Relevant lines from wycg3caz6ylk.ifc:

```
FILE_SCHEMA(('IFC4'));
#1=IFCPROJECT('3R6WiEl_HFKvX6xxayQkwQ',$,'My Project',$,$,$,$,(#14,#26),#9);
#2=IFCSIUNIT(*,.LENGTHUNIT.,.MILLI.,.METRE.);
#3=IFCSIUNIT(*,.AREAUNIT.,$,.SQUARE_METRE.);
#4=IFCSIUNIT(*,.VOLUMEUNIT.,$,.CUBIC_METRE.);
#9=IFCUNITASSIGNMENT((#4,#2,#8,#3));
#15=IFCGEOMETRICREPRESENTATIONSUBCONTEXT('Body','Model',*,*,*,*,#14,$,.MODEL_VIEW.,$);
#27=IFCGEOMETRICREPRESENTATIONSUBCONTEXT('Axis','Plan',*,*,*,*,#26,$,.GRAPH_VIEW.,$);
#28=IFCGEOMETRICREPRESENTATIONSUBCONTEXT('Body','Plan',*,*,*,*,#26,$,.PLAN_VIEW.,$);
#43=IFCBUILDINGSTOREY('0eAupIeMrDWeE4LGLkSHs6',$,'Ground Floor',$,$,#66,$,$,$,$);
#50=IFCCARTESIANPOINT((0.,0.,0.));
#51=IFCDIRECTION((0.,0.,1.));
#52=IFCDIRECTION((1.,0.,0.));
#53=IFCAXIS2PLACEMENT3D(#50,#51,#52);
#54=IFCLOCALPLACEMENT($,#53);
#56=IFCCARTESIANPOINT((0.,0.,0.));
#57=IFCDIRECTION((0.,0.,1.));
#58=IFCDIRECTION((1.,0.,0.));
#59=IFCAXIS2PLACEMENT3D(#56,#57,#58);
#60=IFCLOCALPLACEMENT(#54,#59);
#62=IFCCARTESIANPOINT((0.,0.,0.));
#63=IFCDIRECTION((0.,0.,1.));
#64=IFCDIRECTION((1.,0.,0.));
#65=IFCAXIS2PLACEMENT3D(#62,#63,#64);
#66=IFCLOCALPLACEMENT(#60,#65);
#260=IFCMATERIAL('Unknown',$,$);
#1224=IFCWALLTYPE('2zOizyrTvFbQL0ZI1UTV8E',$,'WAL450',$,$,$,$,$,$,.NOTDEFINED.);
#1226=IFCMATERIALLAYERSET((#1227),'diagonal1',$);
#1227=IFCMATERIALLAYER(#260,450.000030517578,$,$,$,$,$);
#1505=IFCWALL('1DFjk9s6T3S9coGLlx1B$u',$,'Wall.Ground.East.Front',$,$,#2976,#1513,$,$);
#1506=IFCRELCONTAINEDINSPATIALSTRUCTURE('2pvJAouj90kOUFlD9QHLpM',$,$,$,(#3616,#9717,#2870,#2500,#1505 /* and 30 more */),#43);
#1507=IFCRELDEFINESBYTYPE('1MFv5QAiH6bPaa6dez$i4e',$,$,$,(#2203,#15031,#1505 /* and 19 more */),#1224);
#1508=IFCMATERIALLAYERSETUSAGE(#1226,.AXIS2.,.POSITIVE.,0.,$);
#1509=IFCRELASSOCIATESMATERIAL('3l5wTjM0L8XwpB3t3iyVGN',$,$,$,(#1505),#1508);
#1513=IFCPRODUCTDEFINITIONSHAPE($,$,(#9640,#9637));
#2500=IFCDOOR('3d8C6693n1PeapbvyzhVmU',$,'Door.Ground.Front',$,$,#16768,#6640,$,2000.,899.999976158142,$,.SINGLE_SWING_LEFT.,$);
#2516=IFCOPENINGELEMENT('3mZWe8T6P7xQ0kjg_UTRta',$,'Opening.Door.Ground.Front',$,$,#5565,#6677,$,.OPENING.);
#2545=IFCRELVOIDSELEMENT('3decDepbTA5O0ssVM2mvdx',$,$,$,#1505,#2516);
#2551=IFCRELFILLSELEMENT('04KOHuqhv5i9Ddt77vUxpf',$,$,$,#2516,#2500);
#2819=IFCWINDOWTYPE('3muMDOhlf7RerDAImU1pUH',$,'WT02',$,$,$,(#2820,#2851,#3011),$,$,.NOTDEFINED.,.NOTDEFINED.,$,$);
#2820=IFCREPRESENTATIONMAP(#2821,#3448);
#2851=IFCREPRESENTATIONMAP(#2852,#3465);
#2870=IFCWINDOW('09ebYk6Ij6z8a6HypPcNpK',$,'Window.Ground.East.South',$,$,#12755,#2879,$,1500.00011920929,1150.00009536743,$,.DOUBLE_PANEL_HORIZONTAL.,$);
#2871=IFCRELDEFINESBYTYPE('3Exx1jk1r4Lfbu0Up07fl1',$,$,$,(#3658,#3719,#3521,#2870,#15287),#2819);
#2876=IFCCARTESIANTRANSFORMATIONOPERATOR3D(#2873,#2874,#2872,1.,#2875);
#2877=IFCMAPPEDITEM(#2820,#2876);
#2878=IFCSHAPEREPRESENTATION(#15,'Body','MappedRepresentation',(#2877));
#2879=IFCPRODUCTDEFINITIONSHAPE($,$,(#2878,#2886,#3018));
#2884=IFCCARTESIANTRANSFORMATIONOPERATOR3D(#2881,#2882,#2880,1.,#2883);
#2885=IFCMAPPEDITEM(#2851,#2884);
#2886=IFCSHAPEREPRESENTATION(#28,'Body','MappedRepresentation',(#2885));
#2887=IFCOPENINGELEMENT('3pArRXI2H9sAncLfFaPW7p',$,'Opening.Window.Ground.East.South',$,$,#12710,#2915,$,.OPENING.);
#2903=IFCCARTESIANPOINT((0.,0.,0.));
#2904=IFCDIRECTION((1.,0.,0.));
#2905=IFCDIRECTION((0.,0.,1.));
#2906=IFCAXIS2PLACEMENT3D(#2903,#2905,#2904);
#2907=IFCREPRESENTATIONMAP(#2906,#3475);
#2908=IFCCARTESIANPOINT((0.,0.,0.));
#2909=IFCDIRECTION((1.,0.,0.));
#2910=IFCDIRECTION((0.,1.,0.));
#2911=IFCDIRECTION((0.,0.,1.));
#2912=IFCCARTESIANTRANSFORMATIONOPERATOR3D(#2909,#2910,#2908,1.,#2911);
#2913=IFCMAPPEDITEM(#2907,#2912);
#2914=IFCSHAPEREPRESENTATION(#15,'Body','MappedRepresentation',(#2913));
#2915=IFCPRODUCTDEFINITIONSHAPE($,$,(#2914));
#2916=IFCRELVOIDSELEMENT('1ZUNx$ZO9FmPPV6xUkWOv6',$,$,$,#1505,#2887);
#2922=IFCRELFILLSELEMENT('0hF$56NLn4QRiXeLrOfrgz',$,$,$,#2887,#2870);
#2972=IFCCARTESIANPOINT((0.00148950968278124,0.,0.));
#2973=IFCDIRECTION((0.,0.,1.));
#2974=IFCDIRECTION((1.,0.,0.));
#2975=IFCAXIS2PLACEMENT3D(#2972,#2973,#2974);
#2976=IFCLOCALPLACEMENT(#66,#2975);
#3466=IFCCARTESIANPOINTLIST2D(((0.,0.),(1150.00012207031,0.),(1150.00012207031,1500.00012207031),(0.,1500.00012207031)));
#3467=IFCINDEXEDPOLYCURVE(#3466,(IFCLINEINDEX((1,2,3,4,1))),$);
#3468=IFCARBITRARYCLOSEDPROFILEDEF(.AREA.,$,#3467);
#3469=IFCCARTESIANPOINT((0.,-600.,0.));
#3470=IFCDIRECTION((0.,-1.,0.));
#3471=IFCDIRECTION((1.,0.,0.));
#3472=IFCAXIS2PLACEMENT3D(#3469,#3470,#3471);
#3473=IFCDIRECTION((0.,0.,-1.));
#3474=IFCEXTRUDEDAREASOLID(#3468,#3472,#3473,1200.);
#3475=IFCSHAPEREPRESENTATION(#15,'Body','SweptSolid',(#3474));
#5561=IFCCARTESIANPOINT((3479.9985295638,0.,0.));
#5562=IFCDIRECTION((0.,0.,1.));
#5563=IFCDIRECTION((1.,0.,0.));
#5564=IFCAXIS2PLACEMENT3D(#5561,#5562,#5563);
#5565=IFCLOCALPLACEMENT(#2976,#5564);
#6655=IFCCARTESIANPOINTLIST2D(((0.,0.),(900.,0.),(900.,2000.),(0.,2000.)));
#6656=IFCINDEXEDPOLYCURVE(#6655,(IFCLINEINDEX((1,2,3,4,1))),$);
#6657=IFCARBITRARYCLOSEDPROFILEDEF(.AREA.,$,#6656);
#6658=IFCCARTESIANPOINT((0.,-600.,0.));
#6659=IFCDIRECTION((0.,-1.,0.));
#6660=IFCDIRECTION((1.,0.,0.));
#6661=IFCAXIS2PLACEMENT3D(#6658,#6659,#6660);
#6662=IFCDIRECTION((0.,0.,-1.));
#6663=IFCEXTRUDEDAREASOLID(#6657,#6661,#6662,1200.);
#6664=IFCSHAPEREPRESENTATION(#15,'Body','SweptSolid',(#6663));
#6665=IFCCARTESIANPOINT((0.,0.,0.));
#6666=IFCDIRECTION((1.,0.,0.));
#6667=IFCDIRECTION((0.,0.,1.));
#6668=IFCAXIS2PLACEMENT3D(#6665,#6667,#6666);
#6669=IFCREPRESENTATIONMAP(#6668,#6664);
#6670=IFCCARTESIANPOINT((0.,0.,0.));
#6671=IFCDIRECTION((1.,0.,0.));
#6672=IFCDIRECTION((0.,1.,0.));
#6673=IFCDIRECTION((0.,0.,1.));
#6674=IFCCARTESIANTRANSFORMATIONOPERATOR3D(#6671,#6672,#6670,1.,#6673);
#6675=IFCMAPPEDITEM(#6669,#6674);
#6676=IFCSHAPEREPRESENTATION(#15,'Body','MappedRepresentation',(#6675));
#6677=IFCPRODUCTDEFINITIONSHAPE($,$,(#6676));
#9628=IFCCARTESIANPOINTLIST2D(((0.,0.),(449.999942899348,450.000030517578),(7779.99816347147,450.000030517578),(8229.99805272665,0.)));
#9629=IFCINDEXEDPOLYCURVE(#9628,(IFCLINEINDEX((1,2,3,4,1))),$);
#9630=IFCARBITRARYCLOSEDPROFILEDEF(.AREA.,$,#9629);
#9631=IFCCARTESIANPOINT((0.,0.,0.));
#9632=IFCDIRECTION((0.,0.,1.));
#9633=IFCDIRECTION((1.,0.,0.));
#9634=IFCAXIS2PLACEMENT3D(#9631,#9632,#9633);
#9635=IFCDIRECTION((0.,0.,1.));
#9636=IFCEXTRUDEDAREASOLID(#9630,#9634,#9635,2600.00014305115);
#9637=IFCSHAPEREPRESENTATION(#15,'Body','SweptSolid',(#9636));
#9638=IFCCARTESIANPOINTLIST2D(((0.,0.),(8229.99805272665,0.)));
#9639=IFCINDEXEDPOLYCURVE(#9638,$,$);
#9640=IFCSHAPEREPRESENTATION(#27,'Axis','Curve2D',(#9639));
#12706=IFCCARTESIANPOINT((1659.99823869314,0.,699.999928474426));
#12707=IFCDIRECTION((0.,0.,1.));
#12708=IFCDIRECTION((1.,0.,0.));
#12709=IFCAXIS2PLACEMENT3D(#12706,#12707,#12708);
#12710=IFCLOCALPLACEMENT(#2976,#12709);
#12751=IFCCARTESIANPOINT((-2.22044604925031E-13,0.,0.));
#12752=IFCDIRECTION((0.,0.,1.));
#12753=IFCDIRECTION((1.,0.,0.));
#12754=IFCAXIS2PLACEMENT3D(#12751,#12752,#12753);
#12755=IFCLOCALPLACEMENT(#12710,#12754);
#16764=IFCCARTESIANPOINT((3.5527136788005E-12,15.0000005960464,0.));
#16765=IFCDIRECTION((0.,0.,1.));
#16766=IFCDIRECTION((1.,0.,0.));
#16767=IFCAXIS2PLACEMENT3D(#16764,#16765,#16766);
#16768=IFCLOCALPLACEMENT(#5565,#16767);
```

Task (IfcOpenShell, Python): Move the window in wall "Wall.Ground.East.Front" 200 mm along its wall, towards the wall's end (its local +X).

```python
import ifcopenshell
import ifcopenshell.api.geometry
import ifcopenshell.util.placement
import ifcopenshell.util.unit

model = ifcopenshell.open("wycg3caz6ylk.ifc")
unit_scale = ifcopenshell.util.unit.calculate_unit_scale(model)

window = model.by_id(2870)
opening = window.FillsVoids[0].RelatingOpeningElement
wall = opening.VoidsElements[0].RelatingBuildingElement

wall_matrix = ifcopenshell.util.placement.get_local_placement(wall.ObjectPlacement)
shift = wall_matrix[:3, 0] * 0.2 / unit_scale
before = ifcopenshell.util.placement.get_local_placement(window.ObjectPlacement)[:3, 3].copy()

# The window is placed relative to its opening, so it follows when the opening moves.
matrix = ifcopenshell.util.placement.get_local_placement(opening.ObjectPlacement)
matrix[:3, 3] += shift
ifcopenshell.api.geometry.edit_object_placement(
    model, product=opening, matrix=matrix, is_si=False, should_transform_children=True
)

after = ifcopenshell.util.placement.get_local_placement(window.ObjectPlacement)[:3, 3]
print("window moved by", (after - before).round(3) + 0.0)

model.write("wycg3caz6ylk-out.ifc")
```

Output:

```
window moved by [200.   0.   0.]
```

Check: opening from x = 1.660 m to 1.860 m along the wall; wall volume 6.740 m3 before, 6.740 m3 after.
